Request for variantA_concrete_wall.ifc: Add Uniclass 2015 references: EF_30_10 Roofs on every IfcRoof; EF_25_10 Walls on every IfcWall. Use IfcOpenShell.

First a look at what the model holds.

```python
import ifcopenshell

model = ifcopenshell.open("variantA_concrete_wall.ifc")
print(model.schema)
print("classifications:", [c.Name for c in model.by_type("IfcClassification")])
for ifc_class in ("IfcDoor", "IfcRoof", "IfcStair", "IfcWall", "IfcWindow"):
    print(ifc_class, len(model.by_type(ifc_class)))
```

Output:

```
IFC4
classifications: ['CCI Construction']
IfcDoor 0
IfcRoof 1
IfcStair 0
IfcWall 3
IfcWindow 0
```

```python
import ifcopenshell
import ifcopenshell.api.classification

model = ifcopenshell.open("variantA_concrete_wall.ifc")

system = ifcopenshell.api.classification.add_classification(model, classification="Uniclass 2015")

codes = {
    "IfcRoof": ("EF_30_10", "Roofs"),
    "IfcWall": ("EF_25_10", "Walls"),
}
for ifc_class, (code, name) in codes.items():
    products = model.by_type(ifc_class)
    ifcopenshell.api.classification.add_reference(
        model, products=products, classification=system, identification=code, name=name
    )
    print(code, len(products))

model.write("variantA_concrete_wall_v2.ifc")
```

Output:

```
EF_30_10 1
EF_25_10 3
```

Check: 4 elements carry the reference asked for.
